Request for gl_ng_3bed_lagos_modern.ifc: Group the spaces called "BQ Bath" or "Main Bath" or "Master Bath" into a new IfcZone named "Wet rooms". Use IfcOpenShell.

First a look at what the model holds.

```python
import ifcopenshell

model = ifcopenshell.open("gl_ng_3bed_lagos_modern.ifc")
print(model.schema)
seen = {}
for space in model.by_type("IfcSpace"):
    seen[space.LongName] = seen.get(space.LongName, 0) + 1
for name, count in sorted(seen.items(), key=str):
    print(count, "x", name)
print("zones:", [z.Name for z in model.by_type("IfcZone")][:20])
```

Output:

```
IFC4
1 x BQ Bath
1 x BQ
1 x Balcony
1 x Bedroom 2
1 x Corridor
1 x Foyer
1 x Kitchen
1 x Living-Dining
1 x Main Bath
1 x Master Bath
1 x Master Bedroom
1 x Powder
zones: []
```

```python
import ifcopenshell
import ifcopenshell.api.group
import ifcopenshell.api.root

model = ifcopenshell.open("gl_ng_3bed_lagos_modern.ifc")

names = {"BQ Bath", "Main Bath", "Master Bath"}
spaces = [s for s in model.by_type("IfcSpace") if s.LongName in names]

zone = ifcopenshell.api.root.create_entity(model, ifc_class="IfcZone", name="Wet rooms")
ifcopenshell.api.group.assign_group(model, products=spaces, group=zone)
print(len(spaces), "spaces in", zone.Name)

model.write("gl_ng_3bed_lagos_modern_updated.ifc")
```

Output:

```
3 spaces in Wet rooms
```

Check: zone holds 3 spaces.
